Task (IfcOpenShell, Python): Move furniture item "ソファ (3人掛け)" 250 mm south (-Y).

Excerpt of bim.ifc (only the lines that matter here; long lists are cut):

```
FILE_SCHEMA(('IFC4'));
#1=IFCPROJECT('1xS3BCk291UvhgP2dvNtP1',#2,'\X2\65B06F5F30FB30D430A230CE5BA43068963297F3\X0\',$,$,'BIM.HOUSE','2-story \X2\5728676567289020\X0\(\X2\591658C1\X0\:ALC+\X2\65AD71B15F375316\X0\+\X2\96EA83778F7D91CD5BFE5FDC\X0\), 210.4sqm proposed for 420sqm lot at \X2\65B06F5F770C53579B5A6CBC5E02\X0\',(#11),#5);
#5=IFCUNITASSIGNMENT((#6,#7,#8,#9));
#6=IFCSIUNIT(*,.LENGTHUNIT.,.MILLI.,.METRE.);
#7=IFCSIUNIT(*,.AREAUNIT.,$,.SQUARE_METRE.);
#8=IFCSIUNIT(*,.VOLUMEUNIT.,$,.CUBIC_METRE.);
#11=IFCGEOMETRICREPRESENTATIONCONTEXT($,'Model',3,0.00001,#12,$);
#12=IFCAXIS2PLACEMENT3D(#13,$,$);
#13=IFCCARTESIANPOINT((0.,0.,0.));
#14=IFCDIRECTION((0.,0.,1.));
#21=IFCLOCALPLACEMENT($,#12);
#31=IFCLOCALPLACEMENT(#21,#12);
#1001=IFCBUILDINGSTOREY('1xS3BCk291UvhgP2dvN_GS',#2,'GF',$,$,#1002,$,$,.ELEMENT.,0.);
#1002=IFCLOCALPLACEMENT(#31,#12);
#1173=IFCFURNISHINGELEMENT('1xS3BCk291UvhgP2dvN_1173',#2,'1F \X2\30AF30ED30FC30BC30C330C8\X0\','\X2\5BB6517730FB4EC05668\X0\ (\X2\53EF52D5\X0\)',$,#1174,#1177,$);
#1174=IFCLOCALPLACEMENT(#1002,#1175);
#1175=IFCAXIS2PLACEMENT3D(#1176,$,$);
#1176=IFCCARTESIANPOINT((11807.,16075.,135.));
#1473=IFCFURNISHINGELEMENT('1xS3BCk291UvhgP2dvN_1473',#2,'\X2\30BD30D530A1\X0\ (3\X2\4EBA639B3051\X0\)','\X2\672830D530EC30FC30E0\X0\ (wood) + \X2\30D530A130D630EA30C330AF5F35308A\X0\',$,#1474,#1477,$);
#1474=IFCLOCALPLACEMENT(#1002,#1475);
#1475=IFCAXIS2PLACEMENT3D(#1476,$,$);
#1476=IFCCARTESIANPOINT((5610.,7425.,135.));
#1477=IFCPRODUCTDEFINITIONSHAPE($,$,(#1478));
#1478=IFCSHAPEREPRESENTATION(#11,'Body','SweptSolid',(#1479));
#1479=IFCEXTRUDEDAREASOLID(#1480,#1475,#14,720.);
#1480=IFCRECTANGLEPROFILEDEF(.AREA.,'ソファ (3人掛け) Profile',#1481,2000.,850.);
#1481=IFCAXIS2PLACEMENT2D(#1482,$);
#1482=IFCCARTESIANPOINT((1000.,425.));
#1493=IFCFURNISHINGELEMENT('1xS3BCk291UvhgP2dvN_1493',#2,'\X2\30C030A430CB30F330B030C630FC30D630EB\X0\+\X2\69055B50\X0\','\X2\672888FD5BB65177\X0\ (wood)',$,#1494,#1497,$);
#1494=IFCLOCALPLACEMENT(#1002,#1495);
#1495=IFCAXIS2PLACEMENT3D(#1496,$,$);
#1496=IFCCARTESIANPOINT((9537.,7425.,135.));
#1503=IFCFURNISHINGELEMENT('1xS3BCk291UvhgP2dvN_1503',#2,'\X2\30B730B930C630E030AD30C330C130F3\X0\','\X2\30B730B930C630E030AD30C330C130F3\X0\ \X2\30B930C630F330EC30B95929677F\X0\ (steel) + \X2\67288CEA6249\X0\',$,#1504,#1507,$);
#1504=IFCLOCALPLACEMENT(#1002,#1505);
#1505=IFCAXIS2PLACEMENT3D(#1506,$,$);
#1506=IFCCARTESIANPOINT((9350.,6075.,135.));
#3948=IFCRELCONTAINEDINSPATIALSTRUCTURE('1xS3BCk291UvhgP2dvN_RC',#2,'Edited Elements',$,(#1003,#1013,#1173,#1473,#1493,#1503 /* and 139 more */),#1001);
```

```python
import ifcopenshell
import ifcopenshell.api.geometry
import ifcopenshell.util.placement
import ifcopenshell.util.unit

model = ifcopenshell.open("bim.ifc")
unit_scale = ifcopenshell.util.unit.calculate_unit_scale(model)

item = model.by_id(1473)
matrix = ifcopenshell.util.placement.get_local_placement(item.ObjectPlacement)
matrix[1, 3] -= 0.25 / unit_scale
ifcopenshell.api.geometry.edit_object_placement(model, product=item, matrix=matrix, is_si=False)

print(ifcopenshell.util.placement.get_local_placement(item.ObjectPlacement).round(3) + 0.0)

model.write("bim_v2.ifc")
```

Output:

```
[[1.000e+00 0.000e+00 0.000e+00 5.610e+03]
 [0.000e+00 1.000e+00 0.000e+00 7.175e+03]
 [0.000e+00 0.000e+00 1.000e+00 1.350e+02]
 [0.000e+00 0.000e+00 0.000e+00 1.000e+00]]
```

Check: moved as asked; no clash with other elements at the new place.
